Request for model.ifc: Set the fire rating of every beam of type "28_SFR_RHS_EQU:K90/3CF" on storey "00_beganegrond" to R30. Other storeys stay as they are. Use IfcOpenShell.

First a look at what the model holds.

```python
import ifcopenshell
import ifcopenshell.util.element

model = ifcopenshell.open("model.ifc")
print(model.schema)
storey = next(s for s in model.by_type("IfcBuildingStorey") if s.Name == "00_beganegrond")
beams = [e for e in ifcopenshell.util.element.get_decomposition(storey) if e.is_a("IfcBeam")]
seen = {}
for e in beams:
    element_type = ifcopenshell.util.element.get_type(e)
    key = (element_type.Name if element_type != e and element_type else None, ifcopenshell.util.element.get_pset(e, "Pset_BeamCommon", "FireRating"))
    seen[key] = seen.get(key, 0) + 1
for (name, value), count in sorted(seen.items(), key=str):
    print(count, "x", name, "|", value)
```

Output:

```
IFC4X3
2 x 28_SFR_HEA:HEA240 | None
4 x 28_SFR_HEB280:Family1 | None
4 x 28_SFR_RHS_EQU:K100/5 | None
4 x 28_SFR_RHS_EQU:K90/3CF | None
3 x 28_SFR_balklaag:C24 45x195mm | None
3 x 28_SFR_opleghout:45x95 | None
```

```python
import ifcopenshell
import ifcopenshell.api.pset
import ifcopenshell.util.element

model = ifcopenshell.open("model.ifc")

storey = next(s for s in model.by_type("IfcBuildingStorey") if s.Name == "00_beganegrond")
beams = [e for e in ifcopenshell.util.element.get_decomposition(storey) if e.is_a("IfcBeam")]

count = 0
for e in beams:
    element_type = ifcopenshell.util.element.get_type(e)
    if element_type in (None, e) or element_type.Name != "28_SFR_RHS_EQU:K90/3CF":
        continue
    # add_pset returns the element's existing set when there is one.
    pset = ifcopenshell.api.pset.add_pset(model, product=e, name="Pset_BeamCommon")
    ifcopenshell.api.pset.edit_pset(model, pset=pset, properties={"FireRating": "R30"})
    count += 1

print(count, "beams updated")

model.write("model_updated.ifc")
```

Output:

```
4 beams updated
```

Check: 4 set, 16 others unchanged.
